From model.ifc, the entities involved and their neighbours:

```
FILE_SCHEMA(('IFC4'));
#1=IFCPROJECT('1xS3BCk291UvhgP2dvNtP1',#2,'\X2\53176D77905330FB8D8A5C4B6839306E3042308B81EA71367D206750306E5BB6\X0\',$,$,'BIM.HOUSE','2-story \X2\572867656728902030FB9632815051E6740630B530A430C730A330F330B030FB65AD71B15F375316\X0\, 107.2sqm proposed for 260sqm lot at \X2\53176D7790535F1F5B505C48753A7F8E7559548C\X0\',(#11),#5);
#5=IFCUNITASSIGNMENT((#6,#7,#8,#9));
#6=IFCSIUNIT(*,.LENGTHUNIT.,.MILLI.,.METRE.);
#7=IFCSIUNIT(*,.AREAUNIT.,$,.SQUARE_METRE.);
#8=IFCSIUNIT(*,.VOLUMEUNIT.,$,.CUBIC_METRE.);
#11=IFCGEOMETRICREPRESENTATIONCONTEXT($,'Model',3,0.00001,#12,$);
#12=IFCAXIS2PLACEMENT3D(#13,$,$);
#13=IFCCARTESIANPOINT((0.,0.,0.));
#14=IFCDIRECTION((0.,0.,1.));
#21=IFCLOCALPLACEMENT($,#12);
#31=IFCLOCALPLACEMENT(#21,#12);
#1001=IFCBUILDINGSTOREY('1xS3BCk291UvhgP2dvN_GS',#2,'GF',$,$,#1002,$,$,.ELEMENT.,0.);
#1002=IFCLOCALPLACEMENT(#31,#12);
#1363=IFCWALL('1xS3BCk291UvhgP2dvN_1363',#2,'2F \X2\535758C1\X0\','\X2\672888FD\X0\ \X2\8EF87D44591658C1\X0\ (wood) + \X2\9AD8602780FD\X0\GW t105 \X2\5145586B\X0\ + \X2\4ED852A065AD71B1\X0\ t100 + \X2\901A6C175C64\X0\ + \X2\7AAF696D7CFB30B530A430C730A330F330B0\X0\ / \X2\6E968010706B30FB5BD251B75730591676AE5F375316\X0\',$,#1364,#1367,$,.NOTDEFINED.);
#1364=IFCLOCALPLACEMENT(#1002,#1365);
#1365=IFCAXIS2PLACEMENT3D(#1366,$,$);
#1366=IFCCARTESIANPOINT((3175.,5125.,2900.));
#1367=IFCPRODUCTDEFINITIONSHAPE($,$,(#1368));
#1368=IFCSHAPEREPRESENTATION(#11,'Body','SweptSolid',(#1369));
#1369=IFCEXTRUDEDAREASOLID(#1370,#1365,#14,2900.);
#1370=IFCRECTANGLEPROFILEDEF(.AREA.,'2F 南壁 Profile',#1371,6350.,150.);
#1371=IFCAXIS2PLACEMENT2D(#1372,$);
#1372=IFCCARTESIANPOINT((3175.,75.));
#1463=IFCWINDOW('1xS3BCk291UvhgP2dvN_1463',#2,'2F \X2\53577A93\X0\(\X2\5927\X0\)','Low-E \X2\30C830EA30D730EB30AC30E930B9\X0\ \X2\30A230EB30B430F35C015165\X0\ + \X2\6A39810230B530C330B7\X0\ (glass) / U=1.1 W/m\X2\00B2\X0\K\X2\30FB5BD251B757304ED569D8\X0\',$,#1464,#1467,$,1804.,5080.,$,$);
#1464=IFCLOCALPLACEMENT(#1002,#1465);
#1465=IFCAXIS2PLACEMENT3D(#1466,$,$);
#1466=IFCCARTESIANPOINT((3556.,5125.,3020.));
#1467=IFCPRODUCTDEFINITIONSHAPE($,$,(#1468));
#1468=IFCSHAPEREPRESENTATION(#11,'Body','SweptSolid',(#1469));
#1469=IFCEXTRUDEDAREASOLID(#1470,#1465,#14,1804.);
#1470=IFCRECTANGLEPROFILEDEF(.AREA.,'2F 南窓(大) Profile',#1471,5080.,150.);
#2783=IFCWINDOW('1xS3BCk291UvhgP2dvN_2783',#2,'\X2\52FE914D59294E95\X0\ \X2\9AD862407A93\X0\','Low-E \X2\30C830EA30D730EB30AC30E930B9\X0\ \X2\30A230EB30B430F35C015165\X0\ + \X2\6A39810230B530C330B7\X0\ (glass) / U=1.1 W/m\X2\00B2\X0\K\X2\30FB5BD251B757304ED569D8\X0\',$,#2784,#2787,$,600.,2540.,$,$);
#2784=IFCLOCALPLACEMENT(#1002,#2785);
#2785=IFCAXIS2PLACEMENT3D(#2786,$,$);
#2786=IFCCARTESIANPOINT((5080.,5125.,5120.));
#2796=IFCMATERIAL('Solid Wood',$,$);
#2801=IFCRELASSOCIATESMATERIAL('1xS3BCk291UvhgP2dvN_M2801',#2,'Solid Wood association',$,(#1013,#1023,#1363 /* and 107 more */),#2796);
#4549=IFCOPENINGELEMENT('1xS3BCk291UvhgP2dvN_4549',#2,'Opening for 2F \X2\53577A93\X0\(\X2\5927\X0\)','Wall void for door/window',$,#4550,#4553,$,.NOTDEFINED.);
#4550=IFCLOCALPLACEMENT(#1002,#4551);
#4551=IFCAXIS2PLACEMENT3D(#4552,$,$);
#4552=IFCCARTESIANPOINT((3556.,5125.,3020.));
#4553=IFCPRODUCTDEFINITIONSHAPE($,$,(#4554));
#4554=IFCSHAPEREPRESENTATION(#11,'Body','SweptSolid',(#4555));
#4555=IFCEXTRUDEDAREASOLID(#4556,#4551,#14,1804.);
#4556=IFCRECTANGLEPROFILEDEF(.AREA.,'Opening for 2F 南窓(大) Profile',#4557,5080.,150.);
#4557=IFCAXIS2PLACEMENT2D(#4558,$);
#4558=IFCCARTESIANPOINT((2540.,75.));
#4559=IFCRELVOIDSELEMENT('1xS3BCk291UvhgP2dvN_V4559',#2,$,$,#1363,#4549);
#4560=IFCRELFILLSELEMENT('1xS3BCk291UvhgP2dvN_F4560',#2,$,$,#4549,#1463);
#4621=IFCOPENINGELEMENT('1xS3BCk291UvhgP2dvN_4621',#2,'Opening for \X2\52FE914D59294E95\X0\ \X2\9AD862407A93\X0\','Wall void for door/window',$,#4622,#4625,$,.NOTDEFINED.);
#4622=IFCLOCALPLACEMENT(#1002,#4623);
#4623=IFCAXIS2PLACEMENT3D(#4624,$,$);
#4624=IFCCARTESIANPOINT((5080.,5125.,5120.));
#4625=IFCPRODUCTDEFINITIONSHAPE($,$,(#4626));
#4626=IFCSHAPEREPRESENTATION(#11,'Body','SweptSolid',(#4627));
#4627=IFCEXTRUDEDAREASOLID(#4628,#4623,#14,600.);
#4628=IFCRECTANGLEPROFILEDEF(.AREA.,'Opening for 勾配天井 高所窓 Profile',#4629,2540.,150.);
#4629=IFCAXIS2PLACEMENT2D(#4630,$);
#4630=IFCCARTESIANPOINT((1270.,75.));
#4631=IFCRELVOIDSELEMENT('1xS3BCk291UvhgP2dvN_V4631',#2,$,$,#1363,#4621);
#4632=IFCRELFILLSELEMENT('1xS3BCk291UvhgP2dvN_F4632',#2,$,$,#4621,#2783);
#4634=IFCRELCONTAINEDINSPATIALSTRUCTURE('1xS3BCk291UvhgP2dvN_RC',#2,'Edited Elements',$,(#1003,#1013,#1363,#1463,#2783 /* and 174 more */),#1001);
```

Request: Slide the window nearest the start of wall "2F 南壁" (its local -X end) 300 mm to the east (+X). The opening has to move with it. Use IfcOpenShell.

```python
import ifcopenshell
import ifcopenshell.api.geometry
import ifcopenshell.util.placement
import ifcopenshell.util.unit

model = ifcopenshell.open("model.ifc")
unit_scale = ifcopenshell.util.unit.calculate_unit_scale(model)

window = model.by_guid("1xS3BCk291UvhgP2dvN_1463")
opening = window.FillsVoids[0].RelatingOpeningElement
wall = opening.VoidsElements[0].RelatingBuildingElement

wall_matrix = ifcopenshell.util.placement.get_local_placement(wall.ObjectPlacement)
shift = wall_matrix[:3, 0] * 0.3 / unit_scale
before = ifcopenshell.util.placement.get_local_placement(window.ObjectPlacement)[:3, 3].copy()

# The window is not placed relative to its opening, so move both.
for product in (opening, window):
    matrix = ifcopenshell.util.placement.get_local_placement(product.ObjectPlacement)
    matrix[:3, 3] += shift
    ifcopenshell.api.geometry.edit_object_placement(model, product=product, matrix=matrix, is_si=False)

after = ifcopenshell.util.placement.get_local_placement(window.ObjectPlacement)[:3, 3]
print("window moved by", (after - before).round(3) + 0.0)

model.write("model_edited.ifc")
```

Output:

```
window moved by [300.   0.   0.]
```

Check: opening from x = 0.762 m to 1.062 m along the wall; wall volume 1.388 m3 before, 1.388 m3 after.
